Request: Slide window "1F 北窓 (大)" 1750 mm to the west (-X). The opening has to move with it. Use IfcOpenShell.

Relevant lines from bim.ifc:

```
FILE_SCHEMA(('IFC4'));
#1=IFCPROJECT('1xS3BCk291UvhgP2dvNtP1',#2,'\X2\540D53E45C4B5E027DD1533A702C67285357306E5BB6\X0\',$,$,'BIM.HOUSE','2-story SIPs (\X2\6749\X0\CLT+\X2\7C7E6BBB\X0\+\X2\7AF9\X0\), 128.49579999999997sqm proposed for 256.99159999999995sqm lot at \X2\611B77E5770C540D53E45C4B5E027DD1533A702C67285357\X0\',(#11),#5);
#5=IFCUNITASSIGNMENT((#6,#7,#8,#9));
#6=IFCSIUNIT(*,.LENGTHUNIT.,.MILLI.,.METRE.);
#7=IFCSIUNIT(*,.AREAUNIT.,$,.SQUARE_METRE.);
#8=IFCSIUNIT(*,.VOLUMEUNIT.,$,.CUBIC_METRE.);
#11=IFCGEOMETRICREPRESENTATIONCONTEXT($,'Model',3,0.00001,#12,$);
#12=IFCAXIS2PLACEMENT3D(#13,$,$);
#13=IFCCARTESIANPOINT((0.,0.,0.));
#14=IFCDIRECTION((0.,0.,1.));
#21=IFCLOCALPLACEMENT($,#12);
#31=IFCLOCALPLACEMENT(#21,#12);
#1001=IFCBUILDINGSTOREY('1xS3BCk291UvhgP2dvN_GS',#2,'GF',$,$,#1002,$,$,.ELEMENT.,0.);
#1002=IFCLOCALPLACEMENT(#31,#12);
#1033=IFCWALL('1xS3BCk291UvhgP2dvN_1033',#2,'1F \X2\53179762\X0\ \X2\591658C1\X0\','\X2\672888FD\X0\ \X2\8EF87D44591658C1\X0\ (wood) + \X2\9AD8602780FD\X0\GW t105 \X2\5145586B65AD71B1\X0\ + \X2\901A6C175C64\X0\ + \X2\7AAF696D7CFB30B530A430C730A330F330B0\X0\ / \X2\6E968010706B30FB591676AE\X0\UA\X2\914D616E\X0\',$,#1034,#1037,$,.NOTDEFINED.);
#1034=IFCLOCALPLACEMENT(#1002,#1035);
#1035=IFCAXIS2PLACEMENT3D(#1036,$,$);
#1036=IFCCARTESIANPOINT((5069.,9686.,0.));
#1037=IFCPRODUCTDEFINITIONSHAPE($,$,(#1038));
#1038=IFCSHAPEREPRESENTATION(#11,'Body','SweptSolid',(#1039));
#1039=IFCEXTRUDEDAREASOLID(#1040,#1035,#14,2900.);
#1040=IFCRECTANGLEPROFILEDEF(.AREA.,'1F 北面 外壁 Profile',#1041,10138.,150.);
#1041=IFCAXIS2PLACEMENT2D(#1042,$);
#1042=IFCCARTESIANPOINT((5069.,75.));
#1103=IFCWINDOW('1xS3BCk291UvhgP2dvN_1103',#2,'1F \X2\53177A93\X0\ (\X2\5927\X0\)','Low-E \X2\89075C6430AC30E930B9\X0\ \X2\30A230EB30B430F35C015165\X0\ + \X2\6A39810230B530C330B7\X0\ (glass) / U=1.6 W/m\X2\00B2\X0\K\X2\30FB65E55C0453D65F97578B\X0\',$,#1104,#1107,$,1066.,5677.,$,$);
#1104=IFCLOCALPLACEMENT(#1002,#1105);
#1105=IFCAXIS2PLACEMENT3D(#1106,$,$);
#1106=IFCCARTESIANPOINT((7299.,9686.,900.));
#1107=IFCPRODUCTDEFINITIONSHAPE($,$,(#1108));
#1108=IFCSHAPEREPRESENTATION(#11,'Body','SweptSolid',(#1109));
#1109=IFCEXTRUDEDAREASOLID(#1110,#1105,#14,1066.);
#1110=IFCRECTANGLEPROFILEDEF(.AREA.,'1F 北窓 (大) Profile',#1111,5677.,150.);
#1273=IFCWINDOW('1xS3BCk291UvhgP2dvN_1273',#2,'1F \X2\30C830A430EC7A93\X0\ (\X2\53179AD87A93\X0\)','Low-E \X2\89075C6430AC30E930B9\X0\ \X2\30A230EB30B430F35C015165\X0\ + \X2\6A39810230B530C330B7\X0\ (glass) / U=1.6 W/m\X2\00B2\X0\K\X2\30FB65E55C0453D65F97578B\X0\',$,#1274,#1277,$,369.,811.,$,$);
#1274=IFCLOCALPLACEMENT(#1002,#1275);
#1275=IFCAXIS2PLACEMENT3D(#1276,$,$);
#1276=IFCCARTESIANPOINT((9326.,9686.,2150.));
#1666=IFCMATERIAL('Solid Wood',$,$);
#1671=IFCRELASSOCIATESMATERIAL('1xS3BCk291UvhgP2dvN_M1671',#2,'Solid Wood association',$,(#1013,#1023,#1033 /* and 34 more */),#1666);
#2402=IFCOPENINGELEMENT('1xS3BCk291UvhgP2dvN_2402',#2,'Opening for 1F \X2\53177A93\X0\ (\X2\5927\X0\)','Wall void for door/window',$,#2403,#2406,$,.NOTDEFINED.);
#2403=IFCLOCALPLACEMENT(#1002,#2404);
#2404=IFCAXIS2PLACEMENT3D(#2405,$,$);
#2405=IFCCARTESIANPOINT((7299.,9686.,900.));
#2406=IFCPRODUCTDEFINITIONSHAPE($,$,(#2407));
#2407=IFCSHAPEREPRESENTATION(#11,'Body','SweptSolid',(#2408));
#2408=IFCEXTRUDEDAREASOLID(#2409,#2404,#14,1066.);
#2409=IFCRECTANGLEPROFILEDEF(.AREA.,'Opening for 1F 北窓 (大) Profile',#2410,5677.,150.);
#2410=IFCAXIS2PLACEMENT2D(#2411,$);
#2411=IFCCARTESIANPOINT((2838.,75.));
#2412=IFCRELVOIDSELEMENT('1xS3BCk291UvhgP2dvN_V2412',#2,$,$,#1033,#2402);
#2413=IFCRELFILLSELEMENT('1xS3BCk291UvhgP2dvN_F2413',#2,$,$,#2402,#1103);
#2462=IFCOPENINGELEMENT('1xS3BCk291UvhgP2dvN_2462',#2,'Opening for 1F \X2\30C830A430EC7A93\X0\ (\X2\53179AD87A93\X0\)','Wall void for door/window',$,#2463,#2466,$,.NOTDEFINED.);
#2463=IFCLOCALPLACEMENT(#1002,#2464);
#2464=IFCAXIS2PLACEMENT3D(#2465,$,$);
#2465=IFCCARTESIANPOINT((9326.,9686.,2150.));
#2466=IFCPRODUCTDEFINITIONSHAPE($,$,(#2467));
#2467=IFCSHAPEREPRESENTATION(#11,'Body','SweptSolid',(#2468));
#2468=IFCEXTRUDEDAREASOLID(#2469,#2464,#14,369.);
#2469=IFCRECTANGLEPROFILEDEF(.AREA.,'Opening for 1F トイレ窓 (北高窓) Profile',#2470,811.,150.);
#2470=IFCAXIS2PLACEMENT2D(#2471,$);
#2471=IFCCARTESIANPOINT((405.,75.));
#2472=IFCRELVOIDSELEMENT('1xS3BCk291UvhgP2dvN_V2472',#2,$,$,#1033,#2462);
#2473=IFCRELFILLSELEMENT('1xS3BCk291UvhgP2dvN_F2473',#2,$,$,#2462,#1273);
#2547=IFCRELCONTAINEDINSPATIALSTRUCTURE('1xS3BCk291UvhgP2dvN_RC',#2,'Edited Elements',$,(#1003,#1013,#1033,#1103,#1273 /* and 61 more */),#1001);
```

```python
import ifcopenshell
import ifcopenshell.api.geometry
import ifcopenshell.util.placement

model = ifcopenshell.open("bim.ifc")

window = model.by_id(1103)
opening = window.FillsVoids[0].RelatingOpeningElement
wall = opening.VoidsElements[0].RelatingBuildingElement

wall_matrix = ifcopenshell.util.placement.get_local_placement(wall.ObjectPlacement)
shift = wall_matrix[:3, 0] * -1750.0
before = ifcopenshell.util.placement.get_local_placement(window.ObjectPlacement)[:3, 3].copy()

# The window is not placed relative to its opening, so move both.
for product in (opening, window):
    matrix = ifcopenshell.util.placement.get_local_placement(product.ObjectPlacement)
    matrix[:3, 3] += shift
    ifcopenshell.api.geometry.edit_object_placement(model, product=product, matrix=matrix, is_si=False)

after = ifcopenshell.util.placement.get_local_placement(window.ObjectPlacement)[:3, 3]
print("window moved by", (after - before).round(3) + 0.0)

model.write("bim_updated.ifc")
```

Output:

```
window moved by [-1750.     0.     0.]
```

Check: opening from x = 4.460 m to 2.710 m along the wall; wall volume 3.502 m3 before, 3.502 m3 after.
